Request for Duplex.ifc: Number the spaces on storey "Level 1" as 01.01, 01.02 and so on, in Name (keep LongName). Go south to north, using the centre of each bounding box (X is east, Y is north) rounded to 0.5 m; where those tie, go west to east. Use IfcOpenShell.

First a look at what the model holds.

```python
import ifcopenshell
import ifcopenshell.util.element
import ifcopenshell.util.placement

model = ifcopenshell.open("Duplex.ifc")
print(model.schema)
storey = next(s for s in model.by_type("IfcBuildingStorey") if s.Name == "Level 1")
spaces = [e for e in ifcopenshell.util.element.get_decomposition(storey) if e.is_a("IfcSpace")]
for e in sorted(spaces, key=lambda e: e.id()):
    origin = ifcopenshell.util.placement.get_local_placement(e.ObjectPlacement)[:3, 3]
    print(e.id(), e.Name, e.LongName, origin.round(2) + 0.0, sep=" | ")
```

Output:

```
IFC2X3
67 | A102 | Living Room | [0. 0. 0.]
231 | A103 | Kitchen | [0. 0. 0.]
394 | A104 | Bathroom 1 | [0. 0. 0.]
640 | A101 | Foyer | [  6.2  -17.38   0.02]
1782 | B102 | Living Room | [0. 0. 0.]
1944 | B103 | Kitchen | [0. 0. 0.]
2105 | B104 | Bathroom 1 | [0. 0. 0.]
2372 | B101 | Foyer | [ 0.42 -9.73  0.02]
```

```python
import ifcopenshell
import ifcopenshell.geom
import ifcopenshell.util.element
import ifcopenshell.util.shape

model = ifcopenshell.open("Duplex.ifc")
settings = ifcopenshell.geom.settings()
settings.set("use-world-coords", True)


def centre(element):
    shape = ifcopenshell.geom.create_shape(settings, element)
    return ifcopenshell.util.shape.get_bbox_centroid(shape.geometry)


storey = next(s for s in model.by_type("IfcBuildingStorey") if s.Name == "Level 1")
spaces = [e for e in ifcopenshell.util.element.get_decomposition(storey) if e.is_a("IfcSpace")]

# Insertion points can sit at a corner or the storey origin, so sort by the geometry (in metres).
centres = {e: centre(e) for e in spaces}
spaces.sort(key=lambda e: (round(centres[e][1] / 0.5), centres[e][0]))

for i, e in enumerate(spaces, start=1):
    number = f"01.{i:02d}"
    e.Name = number
    print(e.id(), number)

model.write("Duplex_updated.ifc")
```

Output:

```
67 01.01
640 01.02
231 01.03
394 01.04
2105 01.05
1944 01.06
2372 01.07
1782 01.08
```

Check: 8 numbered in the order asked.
